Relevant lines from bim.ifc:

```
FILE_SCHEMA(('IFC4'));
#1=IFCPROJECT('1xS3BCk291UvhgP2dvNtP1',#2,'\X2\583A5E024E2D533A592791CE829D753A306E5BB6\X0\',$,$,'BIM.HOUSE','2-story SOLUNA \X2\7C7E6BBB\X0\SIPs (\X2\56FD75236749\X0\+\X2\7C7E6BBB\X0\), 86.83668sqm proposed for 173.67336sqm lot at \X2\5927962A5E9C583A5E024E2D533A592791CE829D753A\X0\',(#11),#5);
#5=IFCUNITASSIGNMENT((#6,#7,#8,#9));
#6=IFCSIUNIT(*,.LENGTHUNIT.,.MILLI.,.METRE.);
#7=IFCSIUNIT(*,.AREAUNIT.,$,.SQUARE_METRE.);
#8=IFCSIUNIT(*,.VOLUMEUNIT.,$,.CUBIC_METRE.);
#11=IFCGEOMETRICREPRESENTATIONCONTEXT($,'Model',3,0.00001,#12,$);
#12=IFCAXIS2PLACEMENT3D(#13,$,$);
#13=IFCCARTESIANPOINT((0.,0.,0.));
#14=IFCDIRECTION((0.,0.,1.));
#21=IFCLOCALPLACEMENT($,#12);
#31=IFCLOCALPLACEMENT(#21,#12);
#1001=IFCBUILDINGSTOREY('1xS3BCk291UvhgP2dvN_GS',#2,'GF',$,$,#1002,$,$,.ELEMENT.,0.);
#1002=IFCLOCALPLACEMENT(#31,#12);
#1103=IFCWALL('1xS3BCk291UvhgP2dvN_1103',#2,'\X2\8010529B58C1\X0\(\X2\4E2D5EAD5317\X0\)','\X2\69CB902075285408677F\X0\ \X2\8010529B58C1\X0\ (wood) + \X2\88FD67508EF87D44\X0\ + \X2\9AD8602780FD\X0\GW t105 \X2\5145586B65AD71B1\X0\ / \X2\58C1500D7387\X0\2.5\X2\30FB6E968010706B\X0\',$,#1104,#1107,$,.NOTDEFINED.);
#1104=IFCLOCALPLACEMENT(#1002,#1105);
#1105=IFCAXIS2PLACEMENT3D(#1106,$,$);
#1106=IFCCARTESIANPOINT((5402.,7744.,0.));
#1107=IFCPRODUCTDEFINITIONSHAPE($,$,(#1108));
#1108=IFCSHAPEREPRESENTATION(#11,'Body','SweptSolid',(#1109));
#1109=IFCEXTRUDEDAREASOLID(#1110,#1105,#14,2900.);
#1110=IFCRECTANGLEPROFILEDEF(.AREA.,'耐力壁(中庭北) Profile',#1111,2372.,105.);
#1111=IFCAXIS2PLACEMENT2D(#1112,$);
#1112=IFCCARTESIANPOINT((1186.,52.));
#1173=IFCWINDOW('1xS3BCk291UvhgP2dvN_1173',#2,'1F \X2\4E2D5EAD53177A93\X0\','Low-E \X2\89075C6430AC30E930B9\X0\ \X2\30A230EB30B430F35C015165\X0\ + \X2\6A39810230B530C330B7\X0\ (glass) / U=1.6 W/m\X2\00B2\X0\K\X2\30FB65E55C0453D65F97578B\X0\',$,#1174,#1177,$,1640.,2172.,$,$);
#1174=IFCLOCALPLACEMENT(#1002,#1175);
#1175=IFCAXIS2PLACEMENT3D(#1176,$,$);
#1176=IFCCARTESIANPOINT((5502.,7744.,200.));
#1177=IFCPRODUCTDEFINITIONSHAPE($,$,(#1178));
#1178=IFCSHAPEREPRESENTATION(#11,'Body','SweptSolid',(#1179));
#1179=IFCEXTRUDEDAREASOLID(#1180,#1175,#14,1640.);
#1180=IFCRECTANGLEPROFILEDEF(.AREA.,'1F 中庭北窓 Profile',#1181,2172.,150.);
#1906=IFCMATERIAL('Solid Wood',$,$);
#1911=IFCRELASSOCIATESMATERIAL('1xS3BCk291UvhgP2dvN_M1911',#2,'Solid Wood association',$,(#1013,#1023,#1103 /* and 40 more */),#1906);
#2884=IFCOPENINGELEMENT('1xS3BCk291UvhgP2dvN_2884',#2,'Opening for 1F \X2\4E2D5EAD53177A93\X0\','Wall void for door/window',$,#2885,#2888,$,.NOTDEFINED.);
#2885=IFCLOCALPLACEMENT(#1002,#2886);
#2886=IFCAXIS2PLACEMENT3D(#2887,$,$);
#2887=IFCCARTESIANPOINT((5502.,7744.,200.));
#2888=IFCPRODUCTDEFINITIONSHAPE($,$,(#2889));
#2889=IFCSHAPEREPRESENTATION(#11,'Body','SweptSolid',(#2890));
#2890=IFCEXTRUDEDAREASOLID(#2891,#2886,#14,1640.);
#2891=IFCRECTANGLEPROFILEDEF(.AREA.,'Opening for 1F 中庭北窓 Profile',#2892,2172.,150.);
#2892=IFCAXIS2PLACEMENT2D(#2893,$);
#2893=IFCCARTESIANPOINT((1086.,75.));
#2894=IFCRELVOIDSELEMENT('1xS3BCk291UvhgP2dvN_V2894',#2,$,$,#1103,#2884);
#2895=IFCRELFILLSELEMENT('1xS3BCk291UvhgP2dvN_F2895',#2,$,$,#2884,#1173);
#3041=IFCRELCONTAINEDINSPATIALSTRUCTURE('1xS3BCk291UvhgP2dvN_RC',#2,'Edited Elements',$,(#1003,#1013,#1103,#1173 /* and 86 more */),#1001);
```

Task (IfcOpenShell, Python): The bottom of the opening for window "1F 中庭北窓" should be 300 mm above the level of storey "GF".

```python
import numpy as np
import ifcopenshell
import ifcopenshell.api.geometry
import ifcopenshell.geom
import ifcopenshell.util.element
import ifcopenshell.util.placement
import ifcopenshell.util.shape
import ifcopenshell.util.unit

model = ifcopenshell.open("bim.ifc")
unit_scale = ifcopenshell.util.unit.calculate_unit_scale(model)

window = model.by_guid("1xS3BCk291UvhgP2dvN_1173")
opening = window.FillsVoids[0].RelatingOpeningElement
storey = ifcopenshell.util.element.get_container(window, ifc_class="IfcBuildingStorey")
level = ifcopenshell.util.placement.get_local_placement(storey.ObjectPlacement)[2, 3]

# The opening's origin need not be at the sill, so measure its lowest point.
shape = ifcopenshell.geom.create_shape(ifcopenshell.geom.settings(), opening)
bottom = ifcopenshell.util.shape.get_shape_bottom_elevation(shape, shape.geometry) / unit_scale
dz = level + 300.0 - bottom

shift = np.array([0.0, 0.0, dz])
# The window is not placed relative to its opening, so move both.
for product in (opening, window):
    matrix = ifcopenshell.util.placement.get_local_placement(product.ObjectPlacement)
    matrix[:3, 3] += shift
    ifcopenshell.api.geometry.edit_object_placement(model, product=product, matrix=matrix, is_si=False)

print(f"moved by {dz * unit_scale:+.3f} m")

model.write("bim_edited.ifc")
```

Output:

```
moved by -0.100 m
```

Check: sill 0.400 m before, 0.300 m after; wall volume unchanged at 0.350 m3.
